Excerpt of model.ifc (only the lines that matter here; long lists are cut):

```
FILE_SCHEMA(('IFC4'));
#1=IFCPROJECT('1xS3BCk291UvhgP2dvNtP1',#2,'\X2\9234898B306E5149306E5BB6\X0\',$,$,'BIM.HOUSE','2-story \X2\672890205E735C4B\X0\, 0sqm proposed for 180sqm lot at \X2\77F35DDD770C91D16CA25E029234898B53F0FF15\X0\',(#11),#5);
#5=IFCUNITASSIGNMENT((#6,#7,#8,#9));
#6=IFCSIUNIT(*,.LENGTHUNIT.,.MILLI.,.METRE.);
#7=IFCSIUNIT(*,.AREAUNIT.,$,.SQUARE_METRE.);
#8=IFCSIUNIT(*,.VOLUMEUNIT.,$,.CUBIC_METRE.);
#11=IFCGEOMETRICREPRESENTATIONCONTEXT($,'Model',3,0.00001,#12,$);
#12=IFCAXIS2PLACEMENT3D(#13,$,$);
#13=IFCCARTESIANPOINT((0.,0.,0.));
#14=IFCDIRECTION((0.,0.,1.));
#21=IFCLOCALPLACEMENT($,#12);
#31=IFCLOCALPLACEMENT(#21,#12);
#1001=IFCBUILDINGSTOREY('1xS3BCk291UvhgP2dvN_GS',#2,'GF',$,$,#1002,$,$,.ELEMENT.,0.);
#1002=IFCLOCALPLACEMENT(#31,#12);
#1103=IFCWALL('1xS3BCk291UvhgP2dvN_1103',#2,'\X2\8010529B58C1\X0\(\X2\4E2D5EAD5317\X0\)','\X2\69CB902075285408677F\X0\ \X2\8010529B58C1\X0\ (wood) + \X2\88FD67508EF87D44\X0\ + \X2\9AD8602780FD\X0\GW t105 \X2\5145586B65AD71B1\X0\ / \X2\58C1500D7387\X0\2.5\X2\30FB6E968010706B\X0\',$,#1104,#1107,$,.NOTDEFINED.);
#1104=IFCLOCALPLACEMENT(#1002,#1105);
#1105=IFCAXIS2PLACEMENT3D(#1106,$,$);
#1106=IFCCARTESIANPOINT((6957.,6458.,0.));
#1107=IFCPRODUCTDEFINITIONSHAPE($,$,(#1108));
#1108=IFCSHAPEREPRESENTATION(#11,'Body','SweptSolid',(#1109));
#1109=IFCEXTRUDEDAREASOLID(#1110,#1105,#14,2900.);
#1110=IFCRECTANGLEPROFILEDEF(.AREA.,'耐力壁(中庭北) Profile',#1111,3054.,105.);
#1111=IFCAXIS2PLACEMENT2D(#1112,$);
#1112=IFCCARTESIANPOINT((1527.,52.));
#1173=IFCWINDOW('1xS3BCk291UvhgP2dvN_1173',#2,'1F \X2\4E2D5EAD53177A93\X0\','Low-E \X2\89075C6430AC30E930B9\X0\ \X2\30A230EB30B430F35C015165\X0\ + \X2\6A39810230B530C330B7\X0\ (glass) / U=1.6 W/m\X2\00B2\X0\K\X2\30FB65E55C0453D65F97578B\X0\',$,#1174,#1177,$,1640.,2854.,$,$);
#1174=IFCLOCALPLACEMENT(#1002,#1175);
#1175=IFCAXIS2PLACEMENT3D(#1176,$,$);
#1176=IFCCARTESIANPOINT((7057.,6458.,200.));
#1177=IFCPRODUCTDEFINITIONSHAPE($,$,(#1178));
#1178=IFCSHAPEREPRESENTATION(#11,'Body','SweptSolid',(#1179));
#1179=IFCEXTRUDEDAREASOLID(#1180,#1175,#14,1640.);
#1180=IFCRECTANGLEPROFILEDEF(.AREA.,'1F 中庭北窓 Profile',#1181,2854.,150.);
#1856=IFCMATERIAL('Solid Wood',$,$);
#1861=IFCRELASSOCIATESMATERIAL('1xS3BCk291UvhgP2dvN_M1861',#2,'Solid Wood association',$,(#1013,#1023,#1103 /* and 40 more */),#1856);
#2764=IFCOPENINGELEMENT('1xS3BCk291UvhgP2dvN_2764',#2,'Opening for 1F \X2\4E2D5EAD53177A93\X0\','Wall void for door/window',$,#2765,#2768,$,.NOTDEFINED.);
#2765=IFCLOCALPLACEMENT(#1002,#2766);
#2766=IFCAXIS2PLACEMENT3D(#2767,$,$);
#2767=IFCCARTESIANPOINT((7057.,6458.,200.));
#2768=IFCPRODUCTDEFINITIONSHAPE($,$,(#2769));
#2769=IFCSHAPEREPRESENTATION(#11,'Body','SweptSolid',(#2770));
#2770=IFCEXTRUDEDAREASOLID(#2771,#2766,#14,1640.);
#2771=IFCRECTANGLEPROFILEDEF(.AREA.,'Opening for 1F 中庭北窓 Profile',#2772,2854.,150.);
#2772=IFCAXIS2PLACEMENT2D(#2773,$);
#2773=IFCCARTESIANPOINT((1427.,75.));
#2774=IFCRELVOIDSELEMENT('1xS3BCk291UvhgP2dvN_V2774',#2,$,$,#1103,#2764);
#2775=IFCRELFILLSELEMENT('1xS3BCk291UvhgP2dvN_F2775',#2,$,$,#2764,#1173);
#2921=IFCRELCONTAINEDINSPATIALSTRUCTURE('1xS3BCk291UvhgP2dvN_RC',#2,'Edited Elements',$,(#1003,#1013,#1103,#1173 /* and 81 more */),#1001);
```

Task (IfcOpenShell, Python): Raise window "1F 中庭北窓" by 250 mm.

```python
import numpy as np
import ifcopenshell
import ifcopenshell.api.geometry
import ifcopenshell.util.placement
import ifcopenshell.util.unit

model = ifcopenshell.open("model.ifc")
unit_scale = ifcopenshell.util.unit.calculate_unit_scale(model)

window = model.by_guid("1xS3BCk291UvhgP2dvN_1173")
opening = window.FillsVoids[0].RelatingOpeningElement
dz = 250.0

shift = np.array([0.0, 0.0, dz])
# The window is not placed relative to its opening, so move both.
for product in (opening, window):
    matrix = ifcopenshell.util.placement.get_local_placement(product.ObjectPlacement)
    matrix[:3, 3] += shift
    ifcopenshell.api.geometry.edit_object_placement(model, product=product, matrix=matrix, is_si=False)

print(f"moved by {dz * unit_scale:+.3f} m")

model.write("model_edited.ifc")
```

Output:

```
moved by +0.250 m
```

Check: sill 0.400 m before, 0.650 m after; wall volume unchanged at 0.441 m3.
